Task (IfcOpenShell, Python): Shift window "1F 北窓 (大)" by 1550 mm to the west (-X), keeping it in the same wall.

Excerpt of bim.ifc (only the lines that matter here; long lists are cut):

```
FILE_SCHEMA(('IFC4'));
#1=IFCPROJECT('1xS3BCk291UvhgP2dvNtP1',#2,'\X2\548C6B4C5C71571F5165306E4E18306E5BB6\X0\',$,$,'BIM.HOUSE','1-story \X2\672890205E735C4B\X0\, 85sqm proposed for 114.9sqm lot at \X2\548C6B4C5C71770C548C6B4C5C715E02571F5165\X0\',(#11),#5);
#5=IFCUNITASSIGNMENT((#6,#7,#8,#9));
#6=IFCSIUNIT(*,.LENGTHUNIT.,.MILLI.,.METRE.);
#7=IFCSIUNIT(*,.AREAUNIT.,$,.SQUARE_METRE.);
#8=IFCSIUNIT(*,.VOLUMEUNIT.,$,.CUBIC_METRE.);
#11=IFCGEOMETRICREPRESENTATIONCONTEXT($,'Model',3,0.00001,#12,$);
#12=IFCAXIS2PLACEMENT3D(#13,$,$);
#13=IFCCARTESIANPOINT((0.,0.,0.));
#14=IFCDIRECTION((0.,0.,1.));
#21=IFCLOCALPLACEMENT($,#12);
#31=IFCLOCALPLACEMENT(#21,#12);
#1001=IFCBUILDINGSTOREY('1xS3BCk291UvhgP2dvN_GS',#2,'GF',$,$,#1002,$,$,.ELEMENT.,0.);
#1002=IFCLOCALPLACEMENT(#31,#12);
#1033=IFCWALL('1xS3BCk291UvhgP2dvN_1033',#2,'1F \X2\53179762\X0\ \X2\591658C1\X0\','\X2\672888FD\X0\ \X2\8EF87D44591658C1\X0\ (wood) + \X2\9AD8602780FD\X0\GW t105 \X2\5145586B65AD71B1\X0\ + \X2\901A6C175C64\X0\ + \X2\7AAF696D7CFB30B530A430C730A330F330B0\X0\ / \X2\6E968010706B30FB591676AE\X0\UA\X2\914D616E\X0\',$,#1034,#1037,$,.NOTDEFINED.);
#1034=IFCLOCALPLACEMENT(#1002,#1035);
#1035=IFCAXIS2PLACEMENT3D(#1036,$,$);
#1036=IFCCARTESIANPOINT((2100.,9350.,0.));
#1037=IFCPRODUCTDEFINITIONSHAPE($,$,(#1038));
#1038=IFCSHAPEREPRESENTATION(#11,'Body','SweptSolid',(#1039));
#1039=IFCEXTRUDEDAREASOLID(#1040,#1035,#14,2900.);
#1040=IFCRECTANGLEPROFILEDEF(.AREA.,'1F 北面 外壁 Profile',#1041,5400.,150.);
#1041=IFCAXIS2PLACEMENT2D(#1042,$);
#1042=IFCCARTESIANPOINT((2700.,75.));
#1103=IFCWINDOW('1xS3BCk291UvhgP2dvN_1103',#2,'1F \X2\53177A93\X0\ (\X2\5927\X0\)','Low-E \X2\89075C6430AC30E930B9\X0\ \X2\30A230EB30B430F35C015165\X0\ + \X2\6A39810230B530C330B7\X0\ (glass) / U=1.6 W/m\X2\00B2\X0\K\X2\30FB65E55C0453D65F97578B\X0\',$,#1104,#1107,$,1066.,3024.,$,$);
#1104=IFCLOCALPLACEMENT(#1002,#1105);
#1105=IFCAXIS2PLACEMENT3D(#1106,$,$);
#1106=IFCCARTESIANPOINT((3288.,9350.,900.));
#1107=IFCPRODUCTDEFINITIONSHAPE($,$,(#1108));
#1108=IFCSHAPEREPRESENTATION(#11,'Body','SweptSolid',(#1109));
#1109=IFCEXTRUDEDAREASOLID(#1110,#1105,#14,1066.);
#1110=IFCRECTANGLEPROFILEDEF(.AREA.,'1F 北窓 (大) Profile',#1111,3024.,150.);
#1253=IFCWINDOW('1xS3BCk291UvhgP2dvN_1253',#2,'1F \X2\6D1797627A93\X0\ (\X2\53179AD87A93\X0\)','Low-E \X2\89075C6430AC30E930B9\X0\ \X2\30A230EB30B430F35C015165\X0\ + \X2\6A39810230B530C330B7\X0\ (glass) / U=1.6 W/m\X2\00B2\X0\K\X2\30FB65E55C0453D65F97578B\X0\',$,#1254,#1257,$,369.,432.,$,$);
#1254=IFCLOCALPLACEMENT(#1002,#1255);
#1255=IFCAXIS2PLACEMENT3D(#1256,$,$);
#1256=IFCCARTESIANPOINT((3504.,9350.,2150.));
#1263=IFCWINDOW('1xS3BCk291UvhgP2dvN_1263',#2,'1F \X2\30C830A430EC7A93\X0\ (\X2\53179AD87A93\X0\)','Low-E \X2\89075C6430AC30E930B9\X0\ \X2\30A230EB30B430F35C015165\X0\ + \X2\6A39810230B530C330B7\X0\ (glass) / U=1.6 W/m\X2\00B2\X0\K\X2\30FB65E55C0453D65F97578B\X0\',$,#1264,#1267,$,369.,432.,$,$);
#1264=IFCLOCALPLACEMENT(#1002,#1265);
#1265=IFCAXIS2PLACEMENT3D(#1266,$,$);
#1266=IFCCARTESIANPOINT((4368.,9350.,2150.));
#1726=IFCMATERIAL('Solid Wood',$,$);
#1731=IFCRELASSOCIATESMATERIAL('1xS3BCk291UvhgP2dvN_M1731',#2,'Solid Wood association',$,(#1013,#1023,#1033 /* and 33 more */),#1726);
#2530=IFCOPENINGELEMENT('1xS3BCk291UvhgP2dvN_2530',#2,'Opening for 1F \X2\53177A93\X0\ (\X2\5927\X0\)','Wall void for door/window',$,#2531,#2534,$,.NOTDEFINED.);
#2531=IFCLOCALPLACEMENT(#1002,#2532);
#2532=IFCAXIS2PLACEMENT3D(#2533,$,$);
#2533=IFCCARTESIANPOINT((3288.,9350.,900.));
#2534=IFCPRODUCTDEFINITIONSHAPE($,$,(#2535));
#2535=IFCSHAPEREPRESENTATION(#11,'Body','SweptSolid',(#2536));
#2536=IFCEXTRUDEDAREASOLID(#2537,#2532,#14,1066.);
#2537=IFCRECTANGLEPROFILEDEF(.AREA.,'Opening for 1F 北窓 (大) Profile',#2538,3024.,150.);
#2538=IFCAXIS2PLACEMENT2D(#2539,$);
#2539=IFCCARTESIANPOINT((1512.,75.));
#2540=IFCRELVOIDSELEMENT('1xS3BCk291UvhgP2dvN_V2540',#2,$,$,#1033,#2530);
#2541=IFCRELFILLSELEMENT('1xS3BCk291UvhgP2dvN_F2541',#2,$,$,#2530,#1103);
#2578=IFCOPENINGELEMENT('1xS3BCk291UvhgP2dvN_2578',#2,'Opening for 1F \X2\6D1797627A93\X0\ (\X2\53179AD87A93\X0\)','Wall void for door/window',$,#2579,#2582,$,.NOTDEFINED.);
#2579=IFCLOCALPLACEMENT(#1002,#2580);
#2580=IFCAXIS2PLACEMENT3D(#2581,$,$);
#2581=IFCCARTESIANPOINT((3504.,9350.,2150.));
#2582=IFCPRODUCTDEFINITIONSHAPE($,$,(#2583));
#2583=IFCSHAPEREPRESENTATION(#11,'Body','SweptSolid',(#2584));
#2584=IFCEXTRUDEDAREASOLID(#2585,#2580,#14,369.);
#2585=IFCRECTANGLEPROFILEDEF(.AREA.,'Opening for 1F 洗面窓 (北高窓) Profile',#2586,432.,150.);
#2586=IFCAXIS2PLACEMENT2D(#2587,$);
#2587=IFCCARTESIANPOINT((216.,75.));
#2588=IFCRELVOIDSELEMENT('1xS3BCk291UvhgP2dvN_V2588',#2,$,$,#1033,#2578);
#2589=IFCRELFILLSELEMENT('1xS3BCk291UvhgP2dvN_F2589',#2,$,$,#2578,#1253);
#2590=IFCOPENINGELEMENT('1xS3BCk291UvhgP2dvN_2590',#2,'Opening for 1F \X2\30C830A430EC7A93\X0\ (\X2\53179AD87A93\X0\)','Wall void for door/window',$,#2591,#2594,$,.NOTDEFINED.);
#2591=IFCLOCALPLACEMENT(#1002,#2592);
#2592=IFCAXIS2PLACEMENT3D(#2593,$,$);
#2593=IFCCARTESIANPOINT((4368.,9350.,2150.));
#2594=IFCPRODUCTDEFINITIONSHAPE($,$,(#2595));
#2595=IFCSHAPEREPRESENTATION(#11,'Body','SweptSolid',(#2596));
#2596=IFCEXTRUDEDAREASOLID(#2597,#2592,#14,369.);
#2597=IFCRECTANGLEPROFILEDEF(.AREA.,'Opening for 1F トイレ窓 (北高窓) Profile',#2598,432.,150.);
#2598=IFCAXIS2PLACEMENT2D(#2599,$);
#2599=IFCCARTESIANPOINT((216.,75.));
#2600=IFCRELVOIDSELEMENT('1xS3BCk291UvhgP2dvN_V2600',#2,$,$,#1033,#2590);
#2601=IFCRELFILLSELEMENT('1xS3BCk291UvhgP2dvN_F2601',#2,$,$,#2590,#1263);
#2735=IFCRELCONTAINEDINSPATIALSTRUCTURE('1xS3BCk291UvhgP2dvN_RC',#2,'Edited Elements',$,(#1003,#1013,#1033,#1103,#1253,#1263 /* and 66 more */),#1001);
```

```python
import ifcopenshell
import ifcopenshell.api.geometry
import ifcopenshell.util.placement
import ifcopenshell.util.unit

model = ifcopenshell.open("bim.ifc")
unit_scale = ifcopenshell.util.unit.calculate_unit_scale(model)

window = model.by_id(1103)
opening = window.FillsVoids[0].RelatingOpeningElement
wall = opening.VoidsElements[0].RelatingBuildingElement

wall_matrix = ifcopenshell.util.placement.get_local_placement(wall.ObjectPlacement)
shift = wall_matrix[:3, 0] * -1.55 / unit_scale
before = ifcopenshell.util.placement.get_local_placement(window.ObjectPlacement)[:3, 3].copy()

# The window is not placed relative to its opening, so move both.
for product in (opening, window):
    matrix = ifcopenshell.util.placement.get_local_placement(product.ObjectPlacement)
    matrix[:3, 3] += shift
    ifcopenshell.api.geometry.edit_object_placement(model, product=product, matrix=matrix, is_si=False)

after = ifcopenshell.util.placement.get_local_placement(window.ObjectPlacement)[:3, 3]
print("window moved by", (after - before).round(3) + 0.0)

model.write("bim_edited.ifc")
```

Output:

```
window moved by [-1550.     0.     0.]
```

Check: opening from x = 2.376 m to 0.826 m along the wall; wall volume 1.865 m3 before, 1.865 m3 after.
